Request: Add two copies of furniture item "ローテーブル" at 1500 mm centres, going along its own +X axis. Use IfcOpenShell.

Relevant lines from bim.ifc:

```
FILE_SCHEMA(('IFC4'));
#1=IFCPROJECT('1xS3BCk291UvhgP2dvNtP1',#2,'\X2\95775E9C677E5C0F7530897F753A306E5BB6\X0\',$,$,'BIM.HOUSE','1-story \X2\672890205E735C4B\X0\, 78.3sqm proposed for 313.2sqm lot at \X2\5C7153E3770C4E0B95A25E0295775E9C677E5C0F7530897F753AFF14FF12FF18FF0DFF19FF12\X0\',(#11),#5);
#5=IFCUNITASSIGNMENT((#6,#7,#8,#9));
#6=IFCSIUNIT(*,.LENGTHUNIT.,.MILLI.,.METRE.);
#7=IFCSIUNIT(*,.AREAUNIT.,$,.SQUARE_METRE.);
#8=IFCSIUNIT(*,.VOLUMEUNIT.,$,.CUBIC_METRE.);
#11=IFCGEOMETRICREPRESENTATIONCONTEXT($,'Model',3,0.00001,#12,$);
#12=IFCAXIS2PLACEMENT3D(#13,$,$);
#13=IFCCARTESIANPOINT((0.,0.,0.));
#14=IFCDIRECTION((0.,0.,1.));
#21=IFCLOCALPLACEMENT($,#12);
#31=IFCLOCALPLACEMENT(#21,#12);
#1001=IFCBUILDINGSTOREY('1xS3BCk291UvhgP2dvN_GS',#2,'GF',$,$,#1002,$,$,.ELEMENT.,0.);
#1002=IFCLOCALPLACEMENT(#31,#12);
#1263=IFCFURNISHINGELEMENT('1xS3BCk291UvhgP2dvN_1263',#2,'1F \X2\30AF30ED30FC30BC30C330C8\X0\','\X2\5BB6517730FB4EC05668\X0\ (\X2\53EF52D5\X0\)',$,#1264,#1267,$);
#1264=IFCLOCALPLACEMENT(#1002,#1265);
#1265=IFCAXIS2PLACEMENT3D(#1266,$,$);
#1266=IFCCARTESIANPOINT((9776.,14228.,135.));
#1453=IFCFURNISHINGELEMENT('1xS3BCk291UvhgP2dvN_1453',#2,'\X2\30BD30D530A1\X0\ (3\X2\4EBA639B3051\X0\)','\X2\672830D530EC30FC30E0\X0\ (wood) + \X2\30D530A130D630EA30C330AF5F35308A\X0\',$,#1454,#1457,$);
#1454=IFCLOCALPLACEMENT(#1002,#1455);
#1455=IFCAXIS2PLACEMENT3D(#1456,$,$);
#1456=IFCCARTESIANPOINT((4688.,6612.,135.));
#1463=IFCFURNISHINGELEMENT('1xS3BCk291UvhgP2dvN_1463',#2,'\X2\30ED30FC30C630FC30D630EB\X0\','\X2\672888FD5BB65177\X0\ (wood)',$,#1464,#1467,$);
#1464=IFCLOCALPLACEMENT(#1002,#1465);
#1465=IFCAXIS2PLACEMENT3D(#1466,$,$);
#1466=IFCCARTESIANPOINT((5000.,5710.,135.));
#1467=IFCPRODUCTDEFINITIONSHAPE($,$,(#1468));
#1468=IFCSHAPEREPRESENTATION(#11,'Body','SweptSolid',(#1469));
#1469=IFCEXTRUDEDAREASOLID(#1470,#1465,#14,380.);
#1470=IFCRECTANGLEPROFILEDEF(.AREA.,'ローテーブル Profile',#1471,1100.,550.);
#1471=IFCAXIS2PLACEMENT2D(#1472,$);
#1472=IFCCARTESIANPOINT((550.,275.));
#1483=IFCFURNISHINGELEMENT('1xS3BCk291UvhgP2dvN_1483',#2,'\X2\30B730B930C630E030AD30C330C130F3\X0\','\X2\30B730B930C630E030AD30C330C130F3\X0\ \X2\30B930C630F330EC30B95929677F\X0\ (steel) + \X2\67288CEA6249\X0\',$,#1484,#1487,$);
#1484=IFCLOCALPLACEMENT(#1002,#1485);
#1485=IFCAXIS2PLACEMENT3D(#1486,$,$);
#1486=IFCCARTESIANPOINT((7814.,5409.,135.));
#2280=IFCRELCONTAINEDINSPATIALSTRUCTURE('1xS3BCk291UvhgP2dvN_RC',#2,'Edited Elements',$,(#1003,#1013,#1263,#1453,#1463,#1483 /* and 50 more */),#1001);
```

```python
import ifcopenshell
import ifcopenshell.api.geometry
import ifcopenshell.api.root
import ifcopenshell.util.element
import ifcopenshell.util.placement
import ifcopenshell.util.unit

model = ifcopenshell.open("bim.ifc")
unit_scale = ifcopenshell.util.unit.calculate_unit_scale(model)


def reuse_history(source, copy):
    """copy_class also copies each property set's owner history, people and application; keep the originals."""
    for rel in copy.IsDefinedBy:
        if rel.is_a("IfcRelDefinesByProperties") and (history := rel.RelatingPropertyDefinition.OwnerHistory):
            rel.RelatingPropertyDefinition.OwnerHistory = source.OwnerHistory
            ifcopenshell.util.element.remove_deep2(model, history)


source = model.by_id(1463)
base = ifcopenshell.util.placement.get_local_placement(source.ObjectPlacement)
step = base[:3, 0] * 1.5 / unit_scale

for i in range(1, 3):
    copy = ifcopenshell.api.root.copy_class(model, product=source)
    copy.Representation = ifcopenshell.util.element.copy_deep(
        model, source.Representation, exclude=["IfcGeometricRepresentationContext", "IfcRepresentationMap"]
    )
    reuse_history(source, copy)
    matrix = base.copy()
    matrix[:3, 3] += i * step
    print("added at", matrix[:3, 3].round(3) + 0.0)
    ifcopenshell.api.geometry.edit_object_placement(model, product=copy, matrix=matrix, is_si=False)

model.write("bim_rev.ifc")
```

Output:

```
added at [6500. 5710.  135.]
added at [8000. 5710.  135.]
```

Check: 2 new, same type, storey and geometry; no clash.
